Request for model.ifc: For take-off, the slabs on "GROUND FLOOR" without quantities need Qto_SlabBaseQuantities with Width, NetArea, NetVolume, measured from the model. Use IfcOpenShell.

First a look at what the model holds.

```python
import ifcopenshell
import ifcopenshell.util.element
import ifcopenshell.util.unit

model = ifcopenshell.open("model.ifc")
print(model.schema)
for unit_type in ("LENGTHUNIT", "AREAUNIT", "VOLUMEUNIT"):
    print(unit_type, ifcopenshell.util.unit.calculate_unit_scale(model, unit_type))
storey = next(s for s in model.by_type("IfcBuildingStorey") if s.Name == "GROUND FLOOR")
slabs = [e for e in ifcopenshell.util.element.get_decomposition(storey) if e.is_a("IfcSlab")]
for e in sorted(slabs, key=lambda e: e.id()):
    print(e.id(), e.is_a(), e.Name, list(ifcopenshell.util.element.get_psets(e, qtos_only=True)), sep=" | ")
```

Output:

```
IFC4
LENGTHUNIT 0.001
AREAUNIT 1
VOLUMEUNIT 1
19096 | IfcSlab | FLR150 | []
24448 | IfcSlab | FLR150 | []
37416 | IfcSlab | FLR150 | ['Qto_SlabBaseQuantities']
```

```python
import ifcopenshell
import ifcopenshell.api.pset
import ifcopenshell.geom
import ifcopenshell.util.element
import ifcopenshell.util.shape
import ifcopenshell.util.unit

model = ifcopenshell.open("model.ifc")
unit_scale = ifcopenshell.util.unit.calculate_unit_scale(model)
area_scale = ifcopenshell.util.unit.calculate_unit_scale(model, "AREAUNIT")
volume_scale = ifcopenshell.util.unit.calculate_unit_scale(model, "VOLUMEUNIT")
settings = ifcopenshell.geom.settings()

storey = next(s for s in model.by_type("IfcBuildingStorey") if s.Name == "GROUND FLOOR")
slabs = [e for e in ifcopenshell.util.element.get_decomposition(storey) if e.is_a("IfcSlab")]

for e in sorted(slabs, key=lambda e: e.id()):
    if ifcopenshell.util.element.get_psets(e, qtos_only=True, should_inherit=False):
        continue
    # Geometry comes back in metres, in the element's own axes.
    shape = ifcopenshell.geom.create_shape(settings, e)
    values = {
        "Width": ifcopenshell.util.shape.get_z(shape.geometry) / unit_scale,
        "NetArea": ifcopenshell.util.shape.get_footprint_area(shape.geometry) / area_scale,
        "NetVolume": ifcopenshell.util.shape.get_volume(shape.geometry) / volume_scale,
    }
    qto = ifcopenshell.api.pset.add_qto(model, product=e, name="Qto_SlabBaseQuantities")
    ifcopenshell.api.pset.edit_qto(model, qto=qto, properties=values)
    print(e.id(), {k: round(v, 3) for k, v in values.items()})

model.write("model_updated.ifc")
```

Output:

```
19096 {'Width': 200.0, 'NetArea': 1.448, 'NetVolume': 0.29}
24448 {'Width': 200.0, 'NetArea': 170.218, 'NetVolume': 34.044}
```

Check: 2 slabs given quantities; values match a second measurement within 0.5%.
